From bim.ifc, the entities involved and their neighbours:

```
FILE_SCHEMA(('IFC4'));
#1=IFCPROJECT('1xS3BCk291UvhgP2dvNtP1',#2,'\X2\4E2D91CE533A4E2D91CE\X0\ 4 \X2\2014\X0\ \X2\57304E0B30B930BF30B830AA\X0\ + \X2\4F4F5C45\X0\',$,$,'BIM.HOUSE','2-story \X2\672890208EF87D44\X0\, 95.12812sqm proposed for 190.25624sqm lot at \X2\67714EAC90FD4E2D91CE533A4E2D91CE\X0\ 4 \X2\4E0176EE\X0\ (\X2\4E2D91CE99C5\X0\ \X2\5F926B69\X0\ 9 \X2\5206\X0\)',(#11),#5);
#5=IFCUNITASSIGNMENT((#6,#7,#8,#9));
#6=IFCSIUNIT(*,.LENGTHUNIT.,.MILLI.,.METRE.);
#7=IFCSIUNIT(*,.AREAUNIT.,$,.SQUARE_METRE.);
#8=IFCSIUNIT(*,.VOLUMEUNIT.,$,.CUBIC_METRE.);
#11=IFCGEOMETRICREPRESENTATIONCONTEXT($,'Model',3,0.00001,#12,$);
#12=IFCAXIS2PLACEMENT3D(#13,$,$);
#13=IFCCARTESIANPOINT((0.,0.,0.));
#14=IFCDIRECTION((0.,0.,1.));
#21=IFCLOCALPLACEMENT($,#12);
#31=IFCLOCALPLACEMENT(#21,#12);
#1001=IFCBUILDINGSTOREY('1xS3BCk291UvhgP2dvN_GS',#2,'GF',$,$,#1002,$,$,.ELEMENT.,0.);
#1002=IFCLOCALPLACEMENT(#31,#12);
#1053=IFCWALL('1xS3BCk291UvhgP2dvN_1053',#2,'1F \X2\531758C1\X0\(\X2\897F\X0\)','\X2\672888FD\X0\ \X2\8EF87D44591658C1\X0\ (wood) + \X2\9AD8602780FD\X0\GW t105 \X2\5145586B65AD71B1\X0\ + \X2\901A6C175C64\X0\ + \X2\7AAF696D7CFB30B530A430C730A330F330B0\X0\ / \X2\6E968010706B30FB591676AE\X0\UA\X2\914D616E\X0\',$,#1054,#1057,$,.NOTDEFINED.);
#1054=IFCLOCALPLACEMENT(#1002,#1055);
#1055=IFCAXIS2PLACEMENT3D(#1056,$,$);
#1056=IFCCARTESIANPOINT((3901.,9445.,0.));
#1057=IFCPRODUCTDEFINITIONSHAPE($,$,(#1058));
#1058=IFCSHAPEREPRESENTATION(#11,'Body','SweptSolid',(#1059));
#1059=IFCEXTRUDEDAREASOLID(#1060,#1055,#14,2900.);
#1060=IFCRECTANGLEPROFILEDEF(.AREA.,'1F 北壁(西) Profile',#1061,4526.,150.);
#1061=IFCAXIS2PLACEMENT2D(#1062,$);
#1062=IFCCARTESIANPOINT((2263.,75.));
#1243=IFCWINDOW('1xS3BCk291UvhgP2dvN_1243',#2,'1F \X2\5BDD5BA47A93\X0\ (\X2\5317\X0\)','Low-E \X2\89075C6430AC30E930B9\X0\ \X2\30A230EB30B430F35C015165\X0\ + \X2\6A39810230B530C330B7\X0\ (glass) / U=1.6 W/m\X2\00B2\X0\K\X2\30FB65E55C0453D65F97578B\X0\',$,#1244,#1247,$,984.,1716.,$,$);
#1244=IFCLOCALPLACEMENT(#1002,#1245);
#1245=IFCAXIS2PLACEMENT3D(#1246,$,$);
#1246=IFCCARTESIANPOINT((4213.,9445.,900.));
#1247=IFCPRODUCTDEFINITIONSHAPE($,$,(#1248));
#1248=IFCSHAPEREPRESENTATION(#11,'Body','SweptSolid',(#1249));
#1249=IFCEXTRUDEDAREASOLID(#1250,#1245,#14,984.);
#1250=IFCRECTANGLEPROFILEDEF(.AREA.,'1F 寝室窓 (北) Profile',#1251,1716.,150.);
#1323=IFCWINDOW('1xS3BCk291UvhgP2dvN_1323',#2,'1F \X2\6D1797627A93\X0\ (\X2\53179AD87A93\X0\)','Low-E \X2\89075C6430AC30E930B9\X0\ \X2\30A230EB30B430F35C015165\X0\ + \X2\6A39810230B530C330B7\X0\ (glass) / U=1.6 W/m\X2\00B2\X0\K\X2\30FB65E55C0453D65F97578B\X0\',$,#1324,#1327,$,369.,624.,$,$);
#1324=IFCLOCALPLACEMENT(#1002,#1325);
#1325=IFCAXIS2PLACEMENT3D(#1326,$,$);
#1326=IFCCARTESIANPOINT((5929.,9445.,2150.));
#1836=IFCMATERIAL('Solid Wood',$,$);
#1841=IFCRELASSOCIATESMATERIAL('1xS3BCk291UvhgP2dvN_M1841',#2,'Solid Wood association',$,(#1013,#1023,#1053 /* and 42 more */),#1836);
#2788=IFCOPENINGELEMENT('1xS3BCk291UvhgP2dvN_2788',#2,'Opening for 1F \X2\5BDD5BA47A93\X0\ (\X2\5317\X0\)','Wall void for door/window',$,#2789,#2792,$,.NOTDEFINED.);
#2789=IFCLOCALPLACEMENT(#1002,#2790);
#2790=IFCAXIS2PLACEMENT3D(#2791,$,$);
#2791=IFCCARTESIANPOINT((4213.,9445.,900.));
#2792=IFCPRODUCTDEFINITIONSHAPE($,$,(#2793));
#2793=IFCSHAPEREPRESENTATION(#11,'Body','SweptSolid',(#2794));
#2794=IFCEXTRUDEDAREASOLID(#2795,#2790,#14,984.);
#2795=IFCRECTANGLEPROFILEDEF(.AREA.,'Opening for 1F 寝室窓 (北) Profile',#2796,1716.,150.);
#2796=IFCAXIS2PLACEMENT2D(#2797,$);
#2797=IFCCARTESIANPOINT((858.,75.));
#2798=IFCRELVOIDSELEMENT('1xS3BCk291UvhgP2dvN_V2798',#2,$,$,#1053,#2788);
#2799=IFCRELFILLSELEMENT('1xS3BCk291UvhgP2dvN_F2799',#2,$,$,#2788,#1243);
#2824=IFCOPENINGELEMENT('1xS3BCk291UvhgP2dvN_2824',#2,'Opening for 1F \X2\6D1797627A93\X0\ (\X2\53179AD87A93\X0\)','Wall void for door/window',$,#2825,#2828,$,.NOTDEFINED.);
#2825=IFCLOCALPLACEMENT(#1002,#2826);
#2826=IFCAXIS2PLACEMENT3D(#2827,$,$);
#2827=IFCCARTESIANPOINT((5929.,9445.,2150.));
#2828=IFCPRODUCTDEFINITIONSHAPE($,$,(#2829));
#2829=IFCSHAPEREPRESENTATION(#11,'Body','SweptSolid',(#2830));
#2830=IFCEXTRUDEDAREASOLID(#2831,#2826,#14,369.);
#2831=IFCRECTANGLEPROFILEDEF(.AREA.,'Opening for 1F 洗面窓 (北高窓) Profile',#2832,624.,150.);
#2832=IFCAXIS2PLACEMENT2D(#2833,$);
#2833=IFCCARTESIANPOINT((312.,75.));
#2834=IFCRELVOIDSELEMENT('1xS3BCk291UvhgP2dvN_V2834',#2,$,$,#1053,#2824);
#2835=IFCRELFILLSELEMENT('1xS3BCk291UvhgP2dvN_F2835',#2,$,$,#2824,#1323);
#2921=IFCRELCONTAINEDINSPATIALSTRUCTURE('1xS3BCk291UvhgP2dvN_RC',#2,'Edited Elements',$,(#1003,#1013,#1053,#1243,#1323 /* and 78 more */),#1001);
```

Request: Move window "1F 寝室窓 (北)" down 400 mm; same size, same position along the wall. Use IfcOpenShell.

```python
import numpy as np
import ifcopenshell
import ifcopenshell.api.geometry
import ifcopenshell.util.placement
import ifcopenshell.util.unit

model = ifcopenshell.open("bim.ifc")
unit_scale = ifcopenshell.util.unit.calculate_unit_scale(model)

window = model.by_id(1243)
opening = window.FillsVoids[0].RelatingOpeningElement
dz = -400.0

shift = np.array([0.0, 0.0, dz])
# The window is not placed relative to its opening, so move both.
for product in (opening, window):
    matrix = ifcopenshell.util.placement.get_local_placement(product.ObjectPlacement)
    matrix[:3, 3] += shift
    ifcopenshell.api.geometry.edit_object_placement(model, product=product, matrix=matrix, is_si=False)

print(f"moved by {dz * unit_scale:+.3f} m")

model.write("bim_v2.ifc")
```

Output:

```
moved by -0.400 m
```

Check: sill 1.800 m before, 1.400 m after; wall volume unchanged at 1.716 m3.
